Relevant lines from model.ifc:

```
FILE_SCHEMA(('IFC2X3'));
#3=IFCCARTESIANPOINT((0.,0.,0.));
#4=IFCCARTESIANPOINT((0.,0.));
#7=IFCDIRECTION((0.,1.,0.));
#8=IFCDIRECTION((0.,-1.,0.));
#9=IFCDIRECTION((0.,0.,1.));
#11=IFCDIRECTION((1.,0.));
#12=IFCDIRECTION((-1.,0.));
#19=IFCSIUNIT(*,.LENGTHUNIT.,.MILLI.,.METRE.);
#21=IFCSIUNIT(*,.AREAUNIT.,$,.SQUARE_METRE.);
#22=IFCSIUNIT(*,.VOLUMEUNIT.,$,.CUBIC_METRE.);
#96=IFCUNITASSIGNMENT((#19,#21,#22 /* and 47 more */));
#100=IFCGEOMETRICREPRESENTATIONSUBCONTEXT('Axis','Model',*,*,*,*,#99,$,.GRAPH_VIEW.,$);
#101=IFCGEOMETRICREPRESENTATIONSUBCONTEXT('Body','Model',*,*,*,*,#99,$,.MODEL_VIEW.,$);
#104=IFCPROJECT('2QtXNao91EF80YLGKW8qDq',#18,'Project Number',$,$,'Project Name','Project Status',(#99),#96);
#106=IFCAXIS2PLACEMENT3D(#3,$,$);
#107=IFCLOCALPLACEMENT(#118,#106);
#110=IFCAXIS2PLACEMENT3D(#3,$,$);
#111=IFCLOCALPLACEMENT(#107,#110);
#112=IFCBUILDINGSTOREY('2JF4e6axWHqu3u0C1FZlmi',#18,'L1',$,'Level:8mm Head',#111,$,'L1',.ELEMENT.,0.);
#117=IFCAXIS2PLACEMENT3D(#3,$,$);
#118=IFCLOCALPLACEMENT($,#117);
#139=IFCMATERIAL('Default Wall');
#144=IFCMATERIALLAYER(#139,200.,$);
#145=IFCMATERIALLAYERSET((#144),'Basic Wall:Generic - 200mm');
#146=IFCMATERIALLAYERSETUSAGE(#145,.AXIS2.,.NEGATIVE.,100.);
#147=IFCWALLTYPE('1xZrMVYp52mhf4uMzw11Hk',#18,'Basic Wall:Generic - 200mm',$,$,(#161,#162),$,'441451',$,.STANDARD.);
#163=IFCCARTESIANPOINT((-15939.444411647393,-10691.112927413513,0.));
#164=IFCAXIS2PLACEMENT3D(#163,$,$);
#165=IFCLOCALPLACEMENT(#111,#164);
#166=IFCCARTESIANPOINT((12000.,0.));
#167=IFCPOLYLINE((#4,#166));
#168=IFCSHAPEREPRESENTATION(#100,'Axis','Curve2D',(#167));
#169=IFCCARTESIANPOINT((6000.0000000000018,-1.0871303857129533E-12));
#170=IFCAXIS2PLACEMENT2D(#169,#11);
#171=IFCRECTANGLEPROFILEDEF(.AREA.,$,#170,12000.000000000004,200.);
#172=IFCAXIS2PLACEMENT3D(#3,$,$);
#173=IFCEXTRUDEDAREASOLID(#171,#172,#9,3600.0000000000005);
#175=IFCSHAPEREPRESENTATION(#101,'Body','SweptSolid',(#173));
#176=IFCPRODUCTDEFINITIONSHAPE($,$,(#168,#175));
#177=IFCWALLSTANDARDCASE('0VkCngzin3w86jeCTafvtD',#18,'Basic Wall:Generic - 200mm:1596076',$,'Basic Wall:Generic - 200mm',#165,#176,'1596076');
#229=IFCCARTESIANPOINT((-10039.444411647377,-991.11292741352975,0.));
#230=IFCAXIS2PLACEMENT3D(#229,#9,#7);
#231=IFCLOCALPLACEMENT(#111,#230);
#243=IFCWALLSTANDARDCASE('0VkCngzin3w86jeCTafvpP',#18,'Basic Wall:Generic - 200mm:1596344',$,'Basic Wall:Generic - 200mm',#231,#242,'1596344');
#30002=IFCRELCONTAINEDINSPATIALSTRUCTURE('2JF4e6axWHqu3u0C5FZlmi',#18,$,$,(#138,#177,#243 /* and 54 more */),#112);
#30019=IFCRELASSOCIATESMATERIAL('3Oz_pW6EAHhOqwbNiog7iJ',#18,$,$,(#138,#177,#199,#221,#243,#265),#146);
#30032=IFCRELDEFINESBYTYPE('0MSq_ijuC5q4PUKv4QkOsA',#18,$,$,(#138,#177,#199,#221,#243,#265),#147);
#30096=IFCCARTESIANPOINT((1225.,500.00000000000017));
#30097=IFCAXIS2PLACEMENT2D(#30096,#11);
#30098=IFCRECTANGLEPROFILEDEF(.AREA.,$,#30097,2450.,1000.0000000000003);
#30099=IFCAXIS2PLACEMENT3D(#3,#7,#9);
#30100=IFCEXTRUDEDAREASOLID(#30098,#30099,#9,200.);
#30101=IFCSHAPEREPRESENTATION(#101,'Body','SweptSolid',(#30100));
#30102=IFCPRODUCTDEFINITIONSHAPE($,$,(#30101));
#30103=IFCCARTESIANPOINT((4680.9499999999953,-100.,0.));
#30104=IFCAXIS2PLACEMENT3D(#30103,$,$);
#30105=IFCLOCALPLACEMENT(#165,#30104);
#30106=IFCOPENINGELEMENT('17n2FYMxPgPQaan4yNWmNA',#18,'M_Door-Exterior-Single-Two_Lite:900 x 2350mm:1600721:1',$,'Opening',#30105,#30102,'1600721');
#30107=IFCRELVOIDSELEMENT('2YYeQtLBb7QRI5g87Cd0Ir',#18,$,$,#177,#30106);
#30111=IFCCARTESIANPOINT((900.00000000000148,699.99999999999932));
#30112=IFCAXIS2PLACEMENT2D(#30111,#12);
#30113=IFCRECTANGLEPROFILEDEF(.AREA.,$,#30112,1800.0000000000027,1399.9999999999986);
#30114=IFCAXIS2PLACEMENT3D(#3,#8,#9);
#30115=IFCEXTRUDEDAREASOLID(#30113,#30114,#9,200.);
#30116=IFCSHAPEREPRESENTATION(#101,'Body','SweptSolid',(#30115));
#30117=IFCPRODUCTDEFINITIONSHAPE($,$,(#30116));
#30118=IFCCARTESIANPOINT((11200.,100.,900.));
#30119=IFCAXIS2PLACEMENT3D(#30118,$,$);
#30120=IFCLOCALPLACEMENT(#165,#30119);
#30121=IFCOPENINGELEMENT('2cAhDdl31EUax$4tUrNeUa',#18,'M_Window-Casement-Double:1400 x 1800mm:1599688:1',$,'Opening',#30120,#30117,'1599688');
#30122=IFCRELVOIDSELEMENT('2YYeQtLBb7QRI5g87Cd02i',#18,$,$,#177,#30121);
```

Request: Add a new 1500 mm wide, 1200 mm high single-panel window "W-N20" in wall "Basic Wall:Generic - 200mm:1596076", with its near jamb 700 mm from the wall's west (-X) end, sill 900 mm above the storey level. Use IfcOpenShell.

```python
import numpy as np
import ifcopenshell
import ifcopenshell.api.feature
import ifcopenshell.api.geometry
import ifcopenshell.api.root
import ifcopenshell.api.spatial
import ifcopenshell.api.type
import ifcopenshell.geom
import ifcopenshell.util.element
import ifcopenshell.util.placement
import ifcopenshell.util.representation
import ifcopenshell.util.shape
import ifcopenshell.util.unit

model = ifcopenshell.open("model.ifc")
unit_scale = ifcopenshell.util.unit.calculate_unit_scale(model)
settings = ifcopenshell.geom.settings()


def volume(element):
    """Net volume in cubic metres, openings subtracted."""
    shape = ifcopenshell.geom.create_shape(settings, element)
    return ifcopenshell.util.shape.get_volume(shape.geometry)


wall = model.by_guid("0VkCngzin3w86jeCTafvtD")
storey = ifcopenshell.util.element.get_container(wall, ifc_class="IfcBuildingStorey")
context = ifcopenshell.util.representation.get_context(model, "Model", "Body", "MODEL_VIEW")
before = volume(wall)

width, height, from_end, sill = 1.5, 1.2, 0.7, 0.9  # metres

# The wall runs along its own X axis, and the end named is its -X end.
wall_shape = ifcopenshell.geom.create_shape(settings, wall)
x, y, z = ifcopenshell.util.shape.get_vertices(wall_shape.geometry).T
start = x.min() + from_end
face, thickness = float(y.min()), float(y.max() - y.min())
wall_matrix = ifcopenshell.util.placement.get_local_placement(wall.ObjectPlacement)
level = ifcopenshell.util.placement.get_local_placement(storey.ObjectPlacement)[2, 3]


def in_wall(x, y):
    """Placement at x, y metres in the wall's axes, at sill height."""
    matrix = wall_matrix.copy()
    matrix[:, 3] = wall_matrix @ np.array([x / unit_scale, y / unit_scale, 0.0, 1.0])
    matrix[2, 3] = level + sill / unit_scale
    return matrix


# Opening: a box that overshoots both wall faces by 50 mm.
opening = ifcopenshell.api.root.create_entity(model, ifc_class="IfcOpeningElement")
box = ifcopenshell.api.geometry.add_wall_representation(
    model, context=context, length=width, height=height, thickness=thickness + 0.1
)
ifcopenshell.api.geometry.assign_representation(model, product=opening, representation=box)
ifcopenshell.api.geometry.edit_object_placement(model, product=opening, matrix=in_wall(start, face - 0.05), is_si=False)
ifcopenshell.api.feature.add_feature(model, feature=opening, element=wall)

window = ifcopenshell.api.root.create_entity(model, ifc_class="IfcWindow", name="W-N20")
window.OverallWidth, window.OverallHeight = width / unit_scale, height / unit_scale
body = ifcopenshell.api.geometry.add_window_representation(
    model,
    context=context,
    overall_width=window.OverallWidth,
    overall_height=window.OverallHeight,
    partition_type="SINGLE_PANEL",
)
ifcopenshell.api.geometry.assign_representation(model, product=window, representation=body)
ifcopenshell.api.spatial.assign_container(model, products=[window], relating_structure=storey)
fills = ifcopenshell.api.feature.add_filling(model, opening=opening, element=window)
fills.OwnerHistory = window.OwnerHistory  # required in IFC2X3

# IFC2X3 keeps the operation on the window style.
style = ifcopenshell.api.root.create_entity(model, ifc_class="IfcWindowStyle", name="W-N20")
style.OperationType, style.ConstructionType = "SINGLE_PANEL", "NOTDEFINED"
style.ParameterTakesPrecedence = style.Sizeable = False
ifcopenshell.api.type.assign_type(model, related_objects=[window], relating_type=style)

# Centre the window in the wall's thickness.
ifcopenshell.api.geometry.edit_object_placement(model, product=window, matrix=in_wall(start, face), is_si=False)
window_shape = ifcopenshell.geom.create_shape(settings, window)
depth = ifcopenshell.util.shape.get_vertices(window_shape.geometry)[:, 1]
offset = face + thickness / 2 - (depth.min() + depth.max()) / 2
ifcopenshell.api.geometry.edit_object_placement(model, product=window, matrix=in_wall(start, offset), is_si=False)

after = volume(wall)

print(f"wall volume {before:.3f} -> {after:.3f} m3")

model.write("model_edited.ifc")
```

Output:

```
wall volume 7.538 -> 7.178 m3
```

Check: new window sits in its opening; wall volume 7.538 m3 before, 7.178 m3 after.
